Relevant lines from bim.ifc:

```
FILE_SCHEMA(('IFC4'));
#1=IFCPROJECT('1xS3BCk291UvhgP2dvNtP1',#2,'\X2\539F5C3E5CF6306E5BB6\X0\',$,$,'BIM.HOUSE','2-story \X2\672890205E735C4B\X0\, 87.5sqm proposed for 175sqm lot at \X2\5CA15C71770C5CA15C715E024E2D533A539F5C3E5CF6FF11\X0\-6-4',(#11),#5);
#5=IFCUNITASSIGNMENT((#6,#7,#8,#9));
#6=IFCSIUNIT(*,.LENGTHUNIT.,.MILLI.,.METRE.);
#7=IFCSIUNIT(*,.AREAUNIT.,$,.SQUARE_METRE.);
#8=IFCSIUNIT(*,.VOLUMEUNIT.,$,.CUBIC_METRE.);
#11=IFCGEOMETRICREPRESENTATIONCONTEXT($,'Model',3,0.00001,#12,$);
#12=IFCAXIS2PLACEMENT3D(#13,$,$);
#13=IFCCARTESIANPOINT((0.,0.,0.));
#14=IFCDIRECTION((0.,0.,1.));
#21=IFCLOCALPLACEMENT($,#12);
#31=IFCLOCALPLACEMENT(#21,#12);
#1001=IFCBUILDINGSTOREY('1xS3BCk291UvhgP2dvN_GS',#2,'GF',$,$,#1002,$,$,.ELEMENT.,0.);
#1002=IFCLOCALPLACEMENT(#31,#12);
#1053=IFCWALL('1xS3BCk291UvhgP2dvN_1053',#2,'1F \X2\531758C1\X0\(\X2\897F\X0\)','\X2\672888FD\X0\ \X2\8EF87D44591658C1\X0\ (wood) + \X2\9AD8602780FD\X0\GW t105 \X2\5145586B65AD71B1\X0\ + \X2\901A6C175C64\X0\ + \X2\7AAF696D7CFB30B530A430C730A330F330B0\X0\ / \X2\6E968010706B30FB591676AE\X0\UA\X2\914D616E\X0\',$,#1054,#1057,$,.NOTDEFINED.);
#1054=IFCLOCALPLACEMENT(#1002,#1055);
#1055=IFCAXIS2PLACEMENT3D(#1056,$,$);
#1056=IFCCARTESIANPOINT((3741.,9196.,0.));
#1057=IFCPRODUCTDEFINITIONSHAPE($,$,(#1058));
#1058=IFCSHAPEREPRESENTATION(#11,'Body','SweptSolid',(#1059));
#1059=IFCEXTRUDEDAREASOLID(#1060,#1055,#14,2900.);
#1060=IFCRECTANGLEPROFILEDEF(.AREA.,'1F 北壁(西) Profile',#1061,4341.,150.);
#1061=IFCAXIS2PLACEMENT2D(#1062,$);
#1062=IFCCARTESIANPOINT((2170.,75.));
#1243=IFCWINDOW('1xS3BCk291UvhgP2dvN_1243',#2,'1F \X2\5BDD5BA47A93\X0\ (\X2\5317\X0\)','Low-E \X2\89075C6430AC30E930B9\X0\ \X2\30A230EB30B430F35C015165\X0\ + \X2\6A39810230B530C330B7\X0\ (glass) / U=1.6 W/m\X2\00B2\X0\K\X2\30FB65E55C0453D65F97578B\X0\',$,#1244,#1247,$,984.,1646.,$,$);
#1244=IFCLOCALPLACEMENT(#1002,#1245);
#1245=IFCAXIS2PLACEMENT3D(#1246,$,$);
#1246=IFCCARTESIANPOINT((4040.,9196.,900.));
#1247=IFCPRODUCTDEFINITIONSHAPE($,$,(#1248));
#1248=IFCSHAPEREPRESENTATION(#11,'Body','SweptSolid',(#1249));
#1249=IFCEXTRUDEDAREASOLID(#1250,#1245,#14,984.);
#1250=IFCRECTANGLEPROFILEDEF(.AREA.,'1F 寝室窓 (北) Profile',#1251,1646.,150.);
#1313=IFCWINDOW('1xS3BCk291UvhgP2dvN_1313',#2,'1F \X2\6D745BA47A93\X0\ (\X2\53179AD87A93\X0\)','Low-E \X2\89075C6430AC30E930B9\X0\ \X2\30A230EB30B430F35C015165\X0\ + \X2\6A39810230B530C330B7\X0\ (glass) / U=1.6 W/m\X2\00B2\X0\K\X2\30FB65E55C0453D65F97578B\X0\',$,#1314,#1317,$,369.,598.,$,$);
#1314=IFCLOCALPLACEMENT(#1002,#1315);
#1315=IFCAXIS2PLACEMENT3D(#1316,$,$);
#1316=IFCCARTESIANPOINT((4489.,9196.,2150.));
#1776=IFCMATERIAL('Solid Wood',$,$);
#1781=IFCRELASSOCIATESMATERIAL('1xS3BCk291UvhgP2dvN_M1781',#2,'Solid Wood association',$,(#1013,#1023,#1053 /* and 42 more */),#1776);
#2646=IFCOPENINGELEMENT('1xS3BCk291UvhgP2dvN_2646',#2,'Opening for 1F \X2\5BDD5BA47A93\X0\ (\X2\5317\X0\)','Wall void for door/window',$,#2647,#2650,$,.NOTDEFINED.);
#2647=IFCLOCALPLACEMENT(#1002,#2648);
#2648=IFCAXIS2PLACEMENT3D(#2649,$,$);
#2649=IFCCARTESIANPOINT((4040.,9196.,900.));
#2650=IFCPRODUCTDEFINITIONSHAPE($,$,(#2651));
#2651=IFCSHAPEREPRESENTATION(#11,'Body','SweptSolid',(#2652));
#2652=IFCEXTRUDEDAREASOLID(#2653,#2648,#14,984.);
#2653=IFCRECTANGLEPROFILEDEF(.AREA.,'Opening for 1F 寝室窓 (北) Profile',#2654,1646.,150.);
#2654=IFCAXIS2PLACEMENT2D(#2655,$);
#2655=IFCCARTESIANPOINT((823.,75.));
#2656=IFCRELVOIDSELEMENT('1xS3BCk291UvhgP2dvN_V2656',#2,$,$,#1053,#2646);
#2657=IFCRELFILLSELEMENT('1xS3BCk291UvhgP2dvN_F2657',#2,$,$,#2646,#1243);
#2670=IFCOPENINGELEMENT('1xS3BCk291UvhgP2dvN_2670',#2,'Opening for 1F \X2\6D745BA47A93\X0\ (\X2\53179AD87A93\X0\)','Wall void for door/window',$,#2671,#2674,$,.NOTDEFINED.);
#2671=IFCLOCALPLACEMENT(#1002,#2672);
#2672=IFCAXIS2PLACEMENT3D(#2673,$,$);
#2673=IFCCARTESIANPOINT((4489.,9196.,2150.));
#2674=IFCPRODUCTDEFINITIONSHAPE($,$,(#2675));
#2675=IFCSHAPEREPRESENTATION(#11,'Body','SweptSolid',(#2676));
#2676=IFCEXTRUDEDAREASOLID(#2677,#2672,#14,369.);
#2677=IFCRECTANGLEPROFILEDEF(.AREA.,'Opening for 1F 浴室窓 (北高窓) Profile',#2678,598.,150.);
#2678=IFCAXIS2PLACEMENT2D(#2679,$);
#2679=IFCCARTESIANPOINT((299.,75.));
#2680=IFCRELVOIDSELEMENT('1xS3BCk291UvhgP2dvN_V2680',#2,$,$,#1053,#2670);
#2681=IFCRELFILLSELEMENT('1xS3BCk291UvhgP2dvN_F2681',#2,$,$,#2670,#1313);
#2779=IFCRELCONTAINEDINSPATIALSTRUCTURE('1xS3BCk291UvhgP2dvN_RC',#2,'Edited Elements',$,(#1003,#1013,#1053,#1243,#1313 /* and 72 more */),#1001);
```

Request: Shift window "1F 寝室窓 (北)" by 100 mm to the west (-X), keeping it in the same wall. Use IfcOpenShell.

```python
import ifcopenshell
import ifcopenshell.api.geometry
import ifcopenshell.util.placement
import ifcopenshell.util.unit

model = ifcopenshell.open("bim.ifc")
unit_scale = ifcopenshell.util.unit.calculate_unit_scale(model)

window = model.by_id(1243)
opening = window.FillsVoids[0].RelatingOpeningElement
wall = opening.VoidsElements[0].RelatingBuildingElement

wall_matrix = ifcopenshell.util.placement.get_local_placement(wall.ObjectPlacement)
shift = wall_matrix[:3, 0] * -0.1 / unit_scale
before = ifcopenshell.util.placement.get_local_placement(window.ObjectPlacement)[:3, 3].copy()

# The window is not placed relative to its opening, so move both.
for product in (opening, window):
    matrix = ifcopenshell.util.placement.get_local_placement(product.ObjectPlacement)
    matrix[:3, 3] += shift
    ifcopenshell.api.geometry.edit_object_placement(model, product=product, matrix=matrix, is_si=False)

after = ifcopenshell.util.placement.get_local_placement(window.ObjectPlacement)[:3, 3]
print("window moved by", (after - before).round(3) + 0.0)

model.write("bim_rev.ifc")
```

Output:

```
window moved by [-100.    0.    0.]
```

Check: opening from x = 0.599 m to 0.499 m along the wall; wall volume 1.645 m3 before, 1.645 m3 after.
